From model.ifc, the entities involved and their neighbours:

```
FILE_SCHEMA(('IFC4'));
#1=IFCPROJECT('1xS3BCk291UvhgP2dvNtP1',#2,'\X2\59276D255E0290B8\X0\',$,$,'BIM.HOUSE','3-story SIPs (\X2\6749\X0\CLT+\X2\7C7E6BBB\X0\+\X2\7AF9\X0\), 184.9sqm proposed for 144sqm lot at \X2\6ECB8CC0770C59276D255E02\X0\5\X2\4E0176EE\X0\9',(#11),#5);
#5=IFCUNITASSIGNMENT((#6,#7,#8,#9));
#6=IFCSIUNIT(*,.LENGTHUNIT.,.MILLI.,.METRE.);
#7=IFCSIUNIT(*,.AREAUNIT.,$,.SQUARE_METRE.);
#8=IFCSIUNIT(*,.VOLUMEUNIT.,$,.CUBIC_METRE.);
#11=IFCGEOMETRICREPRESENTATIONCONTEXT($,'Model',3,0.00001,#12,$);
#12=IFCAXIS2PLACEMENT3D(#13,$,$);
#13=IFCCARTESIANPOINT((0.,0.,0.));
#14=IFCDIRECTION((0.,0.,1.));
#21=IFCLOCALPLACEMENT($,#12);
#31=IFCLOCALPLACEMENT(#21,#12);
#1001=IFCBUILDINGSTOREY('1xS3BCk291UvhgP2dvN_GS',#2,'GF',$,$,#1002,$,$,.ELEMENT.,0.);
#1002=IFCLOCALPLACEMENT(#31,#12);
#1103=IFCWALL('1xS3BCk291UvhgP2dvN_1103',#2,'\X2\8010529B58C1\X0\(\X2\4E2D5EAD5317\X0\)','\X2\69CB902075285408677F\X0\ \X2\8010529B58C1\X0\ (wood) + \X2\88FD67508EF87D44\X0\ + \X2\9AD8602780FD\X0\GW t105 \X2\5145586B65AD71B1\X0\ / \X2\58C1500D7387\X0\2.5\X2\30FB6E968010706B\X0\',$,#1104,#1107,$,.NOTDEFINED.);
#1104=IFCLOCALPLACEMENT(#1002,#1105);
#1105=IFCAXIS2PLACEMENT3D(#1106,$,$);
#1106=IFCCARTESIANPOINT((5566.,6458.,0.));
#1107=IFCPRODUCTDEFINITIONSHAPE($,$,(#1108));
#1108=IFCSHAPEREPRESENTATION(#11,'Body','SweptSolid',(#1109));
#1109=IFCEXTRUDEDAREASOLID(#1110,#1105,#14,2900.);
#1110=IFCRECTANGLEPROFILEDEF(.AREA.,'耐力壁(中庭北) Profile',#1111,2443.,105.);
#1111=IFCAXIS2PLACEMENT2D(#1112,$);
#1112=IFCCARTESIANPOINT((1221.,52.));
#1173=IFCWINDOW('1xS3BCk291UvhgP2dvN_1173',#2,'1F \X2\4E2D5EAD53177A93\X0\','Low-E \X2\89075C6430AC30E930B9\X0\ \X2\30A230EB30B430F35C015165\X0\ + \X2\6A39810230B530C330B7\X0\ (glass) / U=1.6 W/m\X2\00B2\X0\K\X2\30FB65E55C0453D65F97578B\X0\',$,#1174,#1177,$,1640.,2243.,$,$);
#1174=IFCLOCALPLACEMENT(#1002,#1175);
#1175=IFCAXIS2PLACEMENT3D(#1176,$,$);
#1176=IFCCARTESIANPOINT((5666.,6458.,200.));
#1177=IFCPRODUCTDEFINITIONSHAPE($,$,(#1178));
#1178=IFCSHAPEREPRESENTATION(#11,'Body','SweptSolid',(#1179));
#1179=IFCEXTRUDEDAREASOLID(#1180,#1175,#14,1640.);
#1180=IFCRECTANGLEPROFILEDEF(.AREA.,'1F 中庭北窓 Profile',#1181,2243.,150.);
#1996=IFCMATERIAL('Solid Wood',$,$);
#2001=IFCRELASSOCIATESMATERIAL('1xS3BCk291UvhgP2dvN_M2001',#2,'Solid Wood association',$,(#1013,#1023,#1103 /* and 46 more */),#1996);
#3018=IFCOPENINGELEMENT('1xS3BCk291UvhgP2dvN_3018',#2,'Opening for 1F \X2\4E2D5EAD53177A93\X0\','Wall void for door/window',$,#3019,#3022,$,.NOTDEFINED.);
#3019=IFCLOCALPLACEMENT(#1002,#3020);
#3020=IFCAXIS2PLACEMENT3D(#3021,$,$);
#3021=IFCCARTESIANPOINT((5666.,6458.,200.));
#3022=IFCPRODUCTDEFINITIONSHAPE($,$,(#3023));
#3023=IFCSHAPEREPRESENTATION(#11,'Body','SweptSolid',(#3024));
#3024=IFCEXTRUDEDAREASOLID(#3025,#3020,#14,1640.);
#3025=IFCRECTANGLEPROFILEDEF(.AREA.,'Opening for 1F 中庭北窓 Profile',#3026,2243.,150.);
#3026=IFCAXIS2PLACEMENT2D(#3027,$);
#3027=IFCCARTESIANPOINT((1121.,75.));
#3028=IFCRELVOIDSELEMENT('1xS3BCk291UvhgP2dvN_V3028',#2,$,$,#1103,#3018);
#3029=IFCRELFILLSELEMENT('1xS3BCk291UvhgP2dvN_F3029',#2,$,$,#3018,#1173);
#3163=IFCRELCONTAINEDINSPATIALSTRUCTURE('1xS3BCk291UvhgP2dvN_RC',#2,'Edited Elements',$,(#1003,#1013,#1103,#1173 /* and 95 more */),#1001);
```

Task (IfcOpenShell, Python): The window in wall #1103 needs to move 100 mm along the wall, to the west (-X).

```python
import ifcopenshell
import ifcopenshell.api.geometry
import ifcopenshell.util.placement
import ifcopenshell.util.unit

model = ifcopenshell.open("model.ifc")
unit_scale = ifcopenshell.util.unit.calculate_unit_scale(model)

window = model.by_guid("1xS3BCk291UvhgP2dvN_1173")
opening = window.FillsVoids[0].RelatingOpeningElement
wall = opening.VoidsElements[0].RelatingBuildingElement

wall_matrix = ifcopenshell.util.placement.get_local_placement(wall.ObjectPlacement)
shift = wall_matrix[:3, 0] * -0.1 / unit_scale
before = ifcopenshell.util.placement.get_local_placement(window.ObjectPlacement)[:3, 3].copy()

# The window is not placed relative to its opening, so move both.
for product in (opening, window):
    matrix = ifcopenshell.util.placement.get_local_placement(product.ObjectPlacement)
    matrix[:3, 3] += shift
    ifcopenshell.api.geometry.edit_object_placement(model, product=product, matrix=matrix, is_si=False)

after = ifcopenshell.util.placement.get_local_placement(window.ObjectPlacement)[:3, 3]
print("window moved by", (after - before).round(3) + 0.0)

model.write("model_v2.ifc")
```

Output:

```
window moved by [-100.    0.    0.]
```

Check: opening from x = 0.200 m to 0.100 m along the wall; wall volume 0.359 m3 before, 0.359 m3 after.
